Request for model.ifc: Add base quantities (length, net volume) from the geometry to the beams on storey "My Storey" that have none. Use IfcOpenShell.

First a look at what the model holds.

```python
import ifcopenshell
import ifcopenshell.util.element
import ifcopenshell.util.unit

model = ifcopenshell.open("model.ifc")
print(model.schema)
for unit_type in ("LENGTHUNIT", "AREAUNIT", "VOLUMEUNIT"):
    print(unit_type, ifcopenshell.util.unit.calculate_unit_scale(model, unit_type))
storey = next(s for s in model.by_type("IfcBuildingStorey") if s.Name == "My Storey")
beams = [e for e in ifcopenshell.util.element.get_decomposition(storey) if e.is_a("IfcBeam")]
for e in sorted(beams, key=lambda e: e.id()):
    print(e.id(), e.is_a(), e.Name, list(ifcopenshell.util.element.get_psets(e, qtos_only=True)), sep=" | ")
```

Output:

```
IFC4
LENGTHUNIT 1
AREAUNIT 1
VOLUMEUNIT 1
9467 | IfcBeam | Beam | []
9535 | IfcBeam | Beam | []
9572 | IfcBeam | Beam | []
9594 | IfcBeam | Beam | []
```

```python
import ifcopenshell
import ifcopenshell.api.pset
import ifcopenshell.geom
import ifcopenshell.util.element
import ifcopenshell.util.shape
import ifcopenshell.util.unit

model = ifcopenshell.open("model.ifc")
unit_scale = ifcopenshell.util.unit.calculate_unit_scale(model)
volume_scale = ifcopenshell.util.unit.calculate_unit_scale(model, "VOLUMEUNIT")
settings = ifcopenshell.geom.settings()

storey = next(s for s in model.by_type("IfcBuildingStorey") if s.Name == "My Storey")
beams = [e for e in ifcopenshell.util.element.get_decomposition(storey) if e.is_a("IfcBeam")]

for e in sorted(beams, key=lambda e: e.id()):
    if ifcopenshell.util.element.get_psets(e, qtos_only=True, should_inherit=False):
        continue
    # Geometry comes back in metres, in the element's own axes.
    shape = ifcopenshell.geom.create_shape(settings, e)
    values = {
        "Length": ifcopenshell.util.shape.get_max_xyz(shape.geometry) / unit_scale,
        "NetVolume": ifcopenshell.util.shape.get_volume(shape.geometry) / volume_scale,
    }
    qto = ifcopenshell.api.pset.add_qto(model, product=e, name="Qto_BeamBaseQuantities")
    ifcopenshell.api.pset.edit_qto(model, qto=qto, properties=values)
    print(e.id(), {k: round(v, 3) for k, v in values.items()})

model.write("model_rev.ifc")
```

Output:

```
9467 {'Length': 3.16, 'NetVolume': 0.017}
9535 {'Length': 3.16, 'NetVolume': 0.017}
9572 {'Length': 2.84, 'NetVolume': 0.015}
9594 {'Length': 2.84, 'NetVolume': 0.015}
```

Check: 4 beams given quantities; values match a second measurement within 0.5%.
